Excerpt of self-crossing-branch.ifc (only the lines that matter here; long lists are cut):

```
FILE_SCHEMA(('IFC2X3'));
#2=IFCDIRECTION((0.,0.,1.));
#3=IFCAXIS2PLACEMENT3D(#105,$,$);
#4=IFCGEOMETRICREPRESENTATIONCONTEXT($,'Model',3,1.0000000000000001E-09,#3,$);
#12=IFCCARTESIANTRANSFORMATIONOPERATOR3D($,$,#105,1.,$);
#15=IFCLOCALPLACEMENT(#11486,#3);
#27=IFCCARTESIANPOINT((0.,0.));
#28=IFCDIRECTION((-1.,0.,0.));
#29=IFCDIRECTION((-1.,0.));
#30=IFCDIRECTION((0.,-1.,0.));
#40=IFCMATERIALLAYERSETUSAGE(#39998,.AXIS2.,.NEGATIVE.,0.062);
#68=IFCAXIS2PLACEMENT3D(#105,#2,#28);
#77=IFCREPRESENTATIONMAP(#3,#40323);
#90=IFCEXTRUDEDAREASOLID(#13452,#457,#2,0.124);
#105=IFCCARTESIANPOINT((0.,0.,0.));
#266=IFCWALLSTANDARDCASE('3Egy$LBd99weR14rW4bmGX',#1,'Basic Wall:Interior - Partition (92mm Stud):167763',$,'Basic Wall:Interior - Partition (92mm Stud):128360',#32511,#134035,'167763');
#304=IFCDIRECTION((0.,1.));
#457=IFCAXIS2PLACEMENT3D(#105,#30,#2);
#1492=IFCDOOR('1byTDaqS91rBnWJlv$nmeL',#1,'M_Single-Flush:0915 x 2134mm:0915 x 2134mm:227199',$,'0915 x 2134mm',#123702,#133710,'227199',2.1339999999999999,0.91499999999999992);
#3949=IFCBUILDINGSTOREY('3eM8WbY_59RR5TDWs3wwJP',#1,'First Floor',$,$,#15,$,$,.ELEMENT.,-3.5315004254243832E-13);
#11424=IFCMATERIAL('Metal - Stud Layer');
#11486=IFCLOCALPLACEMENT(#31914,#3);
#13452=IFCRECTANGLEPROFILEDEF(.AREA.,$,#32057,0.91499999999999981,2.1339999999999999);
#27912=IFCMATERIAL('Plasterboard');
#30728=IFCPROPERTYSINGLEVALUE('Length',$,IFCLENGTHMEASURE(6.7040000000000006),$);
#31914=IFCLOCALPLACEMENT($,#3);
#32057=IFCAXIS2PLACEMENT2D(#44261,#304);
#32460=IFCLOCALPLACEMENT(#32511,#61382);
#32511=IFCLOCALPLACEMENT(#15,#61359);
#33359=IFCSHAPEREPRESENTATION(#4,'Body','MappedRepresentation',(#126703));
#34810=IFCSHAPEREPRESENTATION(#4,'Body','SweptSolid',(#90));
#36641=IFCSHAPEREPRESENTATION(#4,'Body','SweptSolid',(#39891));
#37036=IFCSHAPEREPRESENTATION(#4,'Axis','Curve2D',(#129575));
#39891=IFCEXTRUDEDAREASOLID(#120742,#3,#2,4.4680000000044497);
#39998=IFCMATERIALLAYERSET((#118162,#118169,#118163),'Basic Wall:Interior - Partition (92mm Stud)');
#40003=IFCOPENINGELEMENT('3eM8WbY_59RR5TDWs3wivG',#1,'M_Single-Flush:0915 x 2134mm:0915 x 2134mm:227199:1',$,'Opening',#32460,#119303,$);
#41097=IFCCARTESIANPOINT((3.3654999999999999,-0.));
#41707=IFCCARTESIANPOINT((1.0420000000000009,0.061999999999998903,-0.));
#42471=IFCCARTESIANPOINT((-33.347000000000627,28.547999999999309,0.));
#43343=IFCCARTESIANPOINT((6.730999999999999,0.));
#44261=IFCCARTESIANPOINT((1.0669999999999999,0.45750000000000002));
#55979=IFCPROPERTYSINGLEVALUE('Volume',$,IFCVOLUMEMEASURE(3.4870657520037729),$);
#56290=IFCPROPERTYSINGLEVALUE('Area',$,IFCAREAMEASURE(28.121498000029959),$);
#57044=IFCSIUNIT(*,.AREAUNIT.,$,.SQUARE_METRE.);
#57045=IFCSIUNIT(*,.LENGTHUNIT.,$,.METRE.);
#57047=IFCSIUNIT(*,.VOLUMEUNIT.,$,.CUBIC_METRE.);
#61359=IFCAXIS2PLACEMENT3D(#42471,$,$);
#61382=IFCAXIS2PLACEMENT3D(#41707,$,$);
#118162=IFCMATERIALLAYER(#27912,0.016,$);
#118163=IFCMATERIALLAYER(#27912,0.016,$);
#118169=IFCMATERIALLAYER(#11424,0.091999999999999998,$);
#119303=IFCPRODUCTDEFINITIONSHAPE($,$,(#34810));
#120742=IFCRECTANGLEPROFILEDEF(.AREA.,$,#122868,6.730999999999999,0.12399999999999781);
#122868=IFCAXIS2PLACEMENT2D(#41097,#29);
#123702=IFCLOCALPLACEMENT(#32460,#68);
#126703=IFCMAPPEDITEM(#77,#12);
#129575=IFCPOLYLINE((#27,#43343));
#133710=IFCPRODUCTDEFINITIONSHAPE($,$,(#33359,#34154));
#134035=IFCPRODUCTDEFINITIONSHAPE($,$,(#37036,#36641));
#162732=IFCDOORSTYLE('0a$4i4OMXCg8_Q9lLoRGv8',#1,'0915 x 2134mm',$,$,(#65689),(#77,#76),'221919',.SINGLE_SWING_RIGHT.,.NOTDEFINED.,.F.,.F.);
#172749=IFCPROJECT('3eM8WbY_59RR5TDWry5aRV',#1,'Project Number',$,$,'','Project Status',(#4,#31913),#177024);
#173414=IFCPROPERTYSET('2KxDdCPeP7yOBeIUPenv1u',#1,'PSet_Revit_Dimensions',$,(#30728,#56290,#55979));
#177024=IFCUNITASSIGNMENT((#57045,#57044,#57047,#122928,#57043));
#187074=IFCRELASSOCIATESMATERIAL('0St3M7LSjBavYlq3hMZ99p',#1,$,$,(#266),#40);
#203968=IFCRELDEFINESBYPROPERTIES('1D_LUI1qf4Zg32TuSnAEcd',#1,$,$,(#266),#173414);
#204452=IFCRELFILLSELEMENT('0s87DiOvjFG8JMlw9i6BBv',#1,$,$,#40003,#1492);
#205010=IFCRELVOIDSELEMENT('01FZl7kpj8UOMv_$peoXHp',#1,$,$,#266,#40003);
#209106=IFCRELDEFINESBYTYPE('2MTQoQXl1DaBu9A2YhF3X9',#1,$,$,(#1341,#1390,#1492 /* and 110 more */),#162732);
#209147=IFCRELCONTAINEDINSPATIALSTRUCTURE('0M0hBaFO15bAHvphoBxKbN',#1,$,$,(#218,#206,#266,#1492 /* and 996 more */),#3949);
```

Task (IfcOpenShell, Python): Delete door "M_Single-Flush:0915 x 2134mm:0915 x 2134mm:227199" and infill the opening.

```python
import ifcopenshell
import ifcopenshell.api.feature
import ifcopenshell.api.pset
import ifcopenshell.api.root
import ifcopenshell.geom
import ifcopenshell.util.element
import ifcopenshell.util.shape
import ifcopenshell.util.unit

model = ifcopenshell.open("self-crossing-branch.ifc")
area_scale = ifcopenshell.util.unit.calculate_unit_scale(model, "AREAUNIT")
volume_scale = ifcopenshell.util.unit.calculate_unit_scale(model, "VOLUMEUNIT")
settings = ifcopenshell.geom.settings()


def volume(element):
    """Net volume in cubic metres, openings subtracted."""
    shape = ifcopenshell.geom.create_shape(settings, element)
    return ifcopenshell.util.shape.get_volume(shape.geometry)


door = model.by_id(1492)
opening = door.FillsVoids[0].RelatingOpeningElement
wall = opening.VoidsElements[0].RelatingBuildingElement
before = volume(wall)

ifcopenshell.api.root.remove_product(model, product=door)
ifcopenshell.api.feature.remove_feature(model, feature=opening)

after = volume(wall)
thickness = 0.124  # wall thickness in metres

# Update the wall's stored quantities.
pset = model.by_id(ifcopenshell.util.element.get_pset(wall, "PSet_Revit_Dimensions", should_inherit=False)["id"])
ifcopenshell.api.pset.edit_pset(model, pset=pset, properties={
    "Area": model.create_entity("IfcAreaMeasure", after / thickness / area_scale),
    "Volume": model.create_entity("IfcVolumeMeasure", after / volume_scale),
})

print(f"wall volume {before:.3f} -> {after:.3f} m3")

model.write("self-crossing-branch_rev.ifc")
```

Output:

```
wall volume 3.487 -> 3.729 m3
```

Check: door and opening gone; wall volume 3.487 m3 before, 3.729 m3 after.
